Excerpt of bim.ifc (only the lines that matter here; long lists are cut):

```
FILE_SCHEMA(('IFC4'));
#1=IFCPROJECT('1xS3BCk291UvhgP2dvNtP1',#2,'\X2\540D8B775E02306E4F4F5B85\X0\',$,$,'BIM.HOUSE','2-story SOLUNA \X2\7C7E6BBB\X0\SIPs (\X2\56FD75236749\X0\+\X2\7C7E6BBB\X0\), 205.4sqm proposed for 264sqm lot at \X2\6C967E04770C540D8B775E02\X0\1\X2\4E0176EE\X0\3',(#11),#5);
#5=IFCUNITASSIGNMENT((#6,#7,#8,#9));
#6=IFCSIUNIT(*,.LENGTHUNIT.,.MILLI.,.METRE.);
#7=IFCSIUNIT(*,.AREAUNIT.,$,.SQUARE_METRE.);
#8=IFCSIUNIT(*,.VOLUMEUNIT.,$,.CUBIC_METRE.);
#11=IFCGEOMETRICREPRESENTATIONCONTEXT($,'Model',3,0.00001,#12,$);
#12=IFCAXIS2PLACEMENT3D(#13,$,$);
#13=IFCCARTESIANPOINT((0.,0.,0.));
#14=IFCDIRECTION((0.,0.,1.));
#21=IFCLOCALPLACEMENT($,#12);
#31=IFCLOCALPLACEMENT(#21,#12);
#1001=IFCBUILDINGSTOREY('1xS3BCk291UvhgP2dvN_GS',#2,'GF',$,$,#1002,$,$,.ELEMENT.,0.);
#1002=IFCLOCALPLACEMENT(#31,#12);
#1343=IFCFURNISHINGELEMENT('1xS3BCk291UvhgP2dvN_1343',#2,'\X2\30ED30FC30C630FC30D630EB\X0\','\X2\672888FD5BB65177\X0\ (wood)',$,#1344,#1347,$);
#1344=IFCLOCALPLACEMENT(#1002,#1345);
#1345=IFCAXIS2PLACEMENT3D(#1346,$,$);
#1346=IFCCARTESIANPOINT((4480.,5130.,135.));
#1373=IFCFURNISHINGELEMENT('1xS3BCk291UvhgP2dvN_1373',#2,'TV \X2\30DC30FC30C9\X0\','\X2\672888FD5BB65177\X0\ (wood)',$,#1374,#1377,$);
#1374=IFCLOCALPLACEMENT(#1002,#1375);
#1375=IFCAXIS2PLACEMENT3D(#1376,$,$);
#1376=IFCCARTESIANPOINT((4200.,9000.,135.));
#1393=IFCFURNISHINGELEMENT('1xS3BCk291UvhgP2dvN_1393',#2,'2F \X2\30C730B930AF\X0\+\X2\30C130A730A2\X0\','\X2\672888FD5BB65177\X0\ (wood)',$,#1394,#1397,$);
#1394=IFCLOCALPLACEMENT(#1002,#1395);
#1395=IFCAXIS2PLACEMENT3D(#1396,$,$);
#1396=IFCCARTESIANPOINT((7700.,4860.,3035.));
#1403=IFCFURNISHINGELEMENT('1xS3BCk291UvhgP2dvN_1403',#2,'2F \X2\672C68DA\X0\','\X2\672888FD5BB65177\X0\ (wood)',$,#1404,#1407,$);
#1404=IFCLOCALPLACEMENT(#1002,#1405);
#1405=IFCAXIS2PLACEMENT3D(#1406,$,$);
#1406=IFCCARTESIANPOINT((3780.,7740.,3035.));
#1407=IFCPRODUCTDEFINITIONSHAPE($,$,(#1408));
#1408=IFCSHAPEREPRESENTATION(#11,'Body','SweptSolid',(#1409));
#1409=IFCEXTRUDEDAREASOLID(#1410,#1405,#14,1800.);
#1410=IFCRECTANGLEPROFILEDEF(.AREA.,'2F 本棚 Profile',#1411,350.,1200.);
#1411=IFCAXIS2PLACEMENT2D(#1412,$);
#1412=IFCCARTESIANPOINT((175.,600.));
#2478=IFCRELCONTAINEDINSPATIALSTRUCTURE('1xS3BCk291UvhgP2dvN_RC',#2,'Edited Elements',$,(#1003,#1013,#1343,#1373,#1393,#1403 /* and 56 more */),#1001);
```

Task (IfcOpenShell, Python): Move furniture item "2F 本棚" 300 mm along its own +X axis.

```python
import ifcopenshell
import ifcopenshell.api.geometry
import ifcopenshell.util.placement

model = ifcopenshell.open("bim.ifc")

item = model.by_guid("1xS3BCk291UvhgP2dvN_1403")
matrix = ifcopenshell.util.placement.get_local_placement(item.ObjectPlacement)
matrix[:3, 3] += matrix[:3, 0] * 300.0
ifcopenshell.api.geometry.edit_object_placement(model, product=item, matrix=matrix, is_si=False)

print(ifcopenshell.util.placement.get_local_placement(item.ObjectPlacement).round(3) + 0.0)

model.write("bim_v2.ifc")
```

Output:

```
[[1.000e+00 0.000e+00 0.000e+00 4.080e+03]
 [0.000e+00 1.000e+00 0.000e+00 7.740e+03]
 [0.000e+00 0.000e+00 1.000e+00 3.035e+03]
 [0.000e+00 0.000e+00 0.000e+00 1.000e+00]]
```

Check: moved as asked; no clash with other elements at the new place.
